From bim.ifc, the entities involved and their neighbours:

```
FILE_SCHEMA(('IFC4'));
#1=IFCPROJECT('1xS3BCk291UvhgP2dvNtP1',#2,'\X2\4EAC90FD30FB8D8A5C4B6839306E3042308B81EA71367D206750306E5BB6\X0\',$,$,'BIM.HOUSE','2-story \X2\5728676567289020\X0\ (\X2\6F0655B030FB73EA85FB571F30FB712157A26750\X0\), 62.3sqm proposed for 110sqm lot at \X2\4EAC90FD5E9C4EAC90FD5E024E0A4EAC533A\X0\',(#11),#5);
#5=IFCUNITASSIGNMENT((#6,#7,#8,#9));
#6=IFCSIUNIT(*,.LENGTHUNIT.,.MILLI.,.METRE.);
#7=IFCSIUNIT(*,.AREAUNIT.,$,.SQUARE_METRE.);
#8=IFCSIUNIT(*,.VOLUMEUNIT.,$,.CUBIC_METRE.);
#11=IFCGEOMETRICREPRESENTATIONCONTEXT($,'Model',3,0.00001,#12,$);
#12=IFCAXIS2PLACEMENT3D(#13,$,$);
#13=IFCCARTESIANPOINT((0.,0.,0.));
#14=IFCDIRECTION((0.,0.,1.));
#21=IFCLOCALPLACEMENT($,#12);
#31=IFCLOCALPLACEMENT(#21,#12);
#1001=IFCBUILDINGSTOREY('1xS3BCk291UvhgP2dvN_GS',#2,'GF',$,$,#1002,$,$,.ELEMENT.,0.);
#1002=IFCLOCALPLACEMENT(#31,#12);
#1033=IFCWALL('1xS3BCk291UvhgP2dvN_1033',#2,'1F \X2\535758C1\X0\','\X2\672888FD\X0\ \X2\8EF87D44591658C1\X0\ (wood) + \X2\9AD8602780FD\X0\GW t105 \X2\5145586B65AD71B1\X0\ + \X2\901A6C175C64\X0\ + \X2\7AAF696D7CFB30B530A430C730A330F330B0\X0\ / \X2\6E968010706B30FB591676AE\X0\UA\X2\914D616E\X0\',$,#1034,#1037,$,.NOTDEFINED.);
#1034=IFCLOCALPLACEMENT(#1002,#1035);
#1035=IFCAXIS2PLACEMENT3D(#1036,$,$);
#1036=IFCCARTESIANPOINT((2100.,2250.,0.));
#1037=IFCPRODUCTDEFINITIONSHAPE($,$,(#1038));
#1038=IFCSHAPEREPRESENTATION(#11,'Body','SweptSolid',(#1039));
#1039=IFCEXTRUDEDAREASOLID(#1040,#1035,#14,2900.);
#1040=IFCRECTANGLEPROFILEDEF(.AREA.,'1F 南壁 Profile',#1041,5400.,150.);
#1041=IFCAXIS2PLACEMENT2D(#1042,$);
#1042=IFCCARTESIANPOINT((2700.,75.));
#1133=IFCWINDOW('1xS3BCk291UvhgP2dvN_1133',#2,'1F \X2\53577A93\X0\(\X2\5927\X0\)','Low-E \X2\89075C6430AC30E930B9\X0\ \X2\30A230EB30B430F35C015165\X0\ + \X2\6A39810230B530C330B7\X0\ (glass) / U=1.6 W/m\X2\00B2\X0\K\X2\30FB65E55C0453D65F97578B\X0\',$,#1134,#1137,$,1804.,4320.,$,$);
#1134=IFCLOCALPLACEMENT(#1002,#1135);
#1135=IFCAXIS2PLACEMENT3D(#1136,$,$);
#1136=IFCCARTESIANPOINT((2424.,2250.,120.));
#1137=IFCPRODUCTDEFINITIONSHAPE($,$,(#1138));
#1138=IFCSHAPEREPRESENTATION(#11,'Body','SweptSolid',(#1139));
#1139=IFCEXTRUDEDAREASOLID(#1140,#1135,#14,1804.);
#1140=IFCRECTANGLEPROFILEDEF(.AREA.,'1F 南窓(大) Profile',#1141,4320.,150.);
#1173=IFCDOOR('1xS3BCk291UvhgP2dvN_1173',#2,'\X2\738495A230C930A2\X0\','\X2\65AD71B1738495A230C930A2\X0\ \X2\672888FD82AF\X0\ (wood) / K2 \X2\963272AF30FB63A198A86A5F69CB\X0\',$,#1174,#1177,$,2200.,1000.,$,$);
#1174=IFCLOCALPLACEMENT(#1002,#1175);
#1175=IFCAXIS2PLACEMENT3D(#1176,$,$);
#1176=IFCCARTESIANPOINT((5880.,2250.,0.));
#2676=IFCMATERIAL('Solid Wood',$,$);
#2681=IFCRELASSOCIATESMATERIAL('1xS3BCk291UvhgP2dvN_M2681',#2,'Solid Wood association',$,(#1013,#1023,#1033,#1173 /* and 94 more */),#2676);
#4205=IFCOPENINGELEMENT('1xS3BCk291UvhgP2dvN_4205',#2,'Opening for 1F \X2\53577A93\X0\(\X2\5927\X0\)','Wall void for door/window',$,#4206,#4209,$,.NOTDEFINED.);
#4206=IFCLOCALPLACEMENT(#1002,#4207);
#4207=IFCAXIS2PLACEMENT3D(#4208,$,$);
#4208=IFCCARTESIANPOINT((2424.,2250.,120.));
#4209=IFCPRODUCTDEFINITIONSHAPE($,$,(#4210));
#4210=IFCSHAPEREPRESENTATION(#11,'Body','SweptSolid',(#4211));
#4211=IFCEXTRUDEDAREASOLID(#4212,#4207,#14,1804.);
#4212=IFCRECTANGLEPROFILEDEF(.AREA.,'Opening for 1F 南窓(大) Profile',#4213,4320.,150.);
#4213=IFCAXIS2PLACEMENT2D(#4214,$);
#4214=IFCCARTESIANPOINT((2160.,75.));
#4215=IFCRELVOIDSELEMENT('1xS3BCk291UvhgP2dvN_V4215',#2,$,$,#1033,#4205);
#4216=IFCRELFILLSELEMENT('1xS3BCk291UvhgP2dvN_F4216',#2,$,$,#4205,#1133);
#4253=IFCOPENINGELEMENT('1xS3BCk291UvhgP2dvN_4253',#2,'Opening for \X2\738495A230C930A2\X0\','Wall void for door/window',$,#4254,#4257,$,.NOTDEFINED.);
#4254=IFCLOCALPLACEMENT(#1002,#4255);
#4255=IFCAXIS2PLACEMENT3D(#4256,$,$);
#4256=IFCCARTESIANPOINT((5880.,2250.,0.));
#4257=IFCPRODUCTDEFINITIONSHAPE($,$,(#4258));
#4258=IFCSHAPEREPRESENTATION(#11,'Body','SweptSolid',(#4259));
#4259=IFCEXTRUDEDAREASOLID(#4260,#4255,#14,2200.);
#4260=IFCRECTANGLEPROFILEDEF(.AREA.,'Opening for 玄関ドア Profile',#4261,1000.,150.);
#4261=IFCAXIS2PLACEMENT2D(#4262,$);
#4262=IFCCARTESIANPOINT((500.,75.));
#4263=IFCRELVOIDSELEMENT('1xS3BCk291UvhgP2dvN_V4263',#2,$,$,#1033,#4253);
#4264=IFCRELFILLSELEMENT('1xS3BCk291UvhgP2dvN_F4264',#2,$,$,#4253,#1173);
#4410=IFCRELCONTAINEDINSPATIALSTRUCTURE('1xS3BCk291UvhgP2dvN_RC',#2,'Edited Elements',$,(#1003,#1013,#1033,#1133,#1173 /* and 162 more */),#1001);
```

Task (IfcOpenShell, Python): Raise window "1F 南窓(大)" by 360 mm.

```python
import numpy as np
import ifcopenshell
import ifcopenshell.api.geometry
import ifcopenshell.util.placement
import ifcopenshell.util.unit

model = ifcopenshell.open("bim.ifc")
unit_scale = ifcopenshell.util.unit.calculate_unit_scale(model)

window = model.by_guid("1xS3BCk291UvhgP2dvN_1133")
opening = window.FillsVoids[0].RelatingOpeningElement
dz = 360.0

shift = np.array([0.0, 0.0, dz])
# The window is not placed relative to its opening, so move both.
for product in (opening, window):
    matrix = ifcopenshell.util.placement.get_local_placement(product.ObjectPlacement)
    matrix[:3, 3] += shift
    ifcopenshell.api.geometry.edit_object_placement(model, product=product, matrix=matrix, is_si=False)

print(f"moved by {dz * unit_scale:+.3f} m")

model.write("bim_rev.ifc")
```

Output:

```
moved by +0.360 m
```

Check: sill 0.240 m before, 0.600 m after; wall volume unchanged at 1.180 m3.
